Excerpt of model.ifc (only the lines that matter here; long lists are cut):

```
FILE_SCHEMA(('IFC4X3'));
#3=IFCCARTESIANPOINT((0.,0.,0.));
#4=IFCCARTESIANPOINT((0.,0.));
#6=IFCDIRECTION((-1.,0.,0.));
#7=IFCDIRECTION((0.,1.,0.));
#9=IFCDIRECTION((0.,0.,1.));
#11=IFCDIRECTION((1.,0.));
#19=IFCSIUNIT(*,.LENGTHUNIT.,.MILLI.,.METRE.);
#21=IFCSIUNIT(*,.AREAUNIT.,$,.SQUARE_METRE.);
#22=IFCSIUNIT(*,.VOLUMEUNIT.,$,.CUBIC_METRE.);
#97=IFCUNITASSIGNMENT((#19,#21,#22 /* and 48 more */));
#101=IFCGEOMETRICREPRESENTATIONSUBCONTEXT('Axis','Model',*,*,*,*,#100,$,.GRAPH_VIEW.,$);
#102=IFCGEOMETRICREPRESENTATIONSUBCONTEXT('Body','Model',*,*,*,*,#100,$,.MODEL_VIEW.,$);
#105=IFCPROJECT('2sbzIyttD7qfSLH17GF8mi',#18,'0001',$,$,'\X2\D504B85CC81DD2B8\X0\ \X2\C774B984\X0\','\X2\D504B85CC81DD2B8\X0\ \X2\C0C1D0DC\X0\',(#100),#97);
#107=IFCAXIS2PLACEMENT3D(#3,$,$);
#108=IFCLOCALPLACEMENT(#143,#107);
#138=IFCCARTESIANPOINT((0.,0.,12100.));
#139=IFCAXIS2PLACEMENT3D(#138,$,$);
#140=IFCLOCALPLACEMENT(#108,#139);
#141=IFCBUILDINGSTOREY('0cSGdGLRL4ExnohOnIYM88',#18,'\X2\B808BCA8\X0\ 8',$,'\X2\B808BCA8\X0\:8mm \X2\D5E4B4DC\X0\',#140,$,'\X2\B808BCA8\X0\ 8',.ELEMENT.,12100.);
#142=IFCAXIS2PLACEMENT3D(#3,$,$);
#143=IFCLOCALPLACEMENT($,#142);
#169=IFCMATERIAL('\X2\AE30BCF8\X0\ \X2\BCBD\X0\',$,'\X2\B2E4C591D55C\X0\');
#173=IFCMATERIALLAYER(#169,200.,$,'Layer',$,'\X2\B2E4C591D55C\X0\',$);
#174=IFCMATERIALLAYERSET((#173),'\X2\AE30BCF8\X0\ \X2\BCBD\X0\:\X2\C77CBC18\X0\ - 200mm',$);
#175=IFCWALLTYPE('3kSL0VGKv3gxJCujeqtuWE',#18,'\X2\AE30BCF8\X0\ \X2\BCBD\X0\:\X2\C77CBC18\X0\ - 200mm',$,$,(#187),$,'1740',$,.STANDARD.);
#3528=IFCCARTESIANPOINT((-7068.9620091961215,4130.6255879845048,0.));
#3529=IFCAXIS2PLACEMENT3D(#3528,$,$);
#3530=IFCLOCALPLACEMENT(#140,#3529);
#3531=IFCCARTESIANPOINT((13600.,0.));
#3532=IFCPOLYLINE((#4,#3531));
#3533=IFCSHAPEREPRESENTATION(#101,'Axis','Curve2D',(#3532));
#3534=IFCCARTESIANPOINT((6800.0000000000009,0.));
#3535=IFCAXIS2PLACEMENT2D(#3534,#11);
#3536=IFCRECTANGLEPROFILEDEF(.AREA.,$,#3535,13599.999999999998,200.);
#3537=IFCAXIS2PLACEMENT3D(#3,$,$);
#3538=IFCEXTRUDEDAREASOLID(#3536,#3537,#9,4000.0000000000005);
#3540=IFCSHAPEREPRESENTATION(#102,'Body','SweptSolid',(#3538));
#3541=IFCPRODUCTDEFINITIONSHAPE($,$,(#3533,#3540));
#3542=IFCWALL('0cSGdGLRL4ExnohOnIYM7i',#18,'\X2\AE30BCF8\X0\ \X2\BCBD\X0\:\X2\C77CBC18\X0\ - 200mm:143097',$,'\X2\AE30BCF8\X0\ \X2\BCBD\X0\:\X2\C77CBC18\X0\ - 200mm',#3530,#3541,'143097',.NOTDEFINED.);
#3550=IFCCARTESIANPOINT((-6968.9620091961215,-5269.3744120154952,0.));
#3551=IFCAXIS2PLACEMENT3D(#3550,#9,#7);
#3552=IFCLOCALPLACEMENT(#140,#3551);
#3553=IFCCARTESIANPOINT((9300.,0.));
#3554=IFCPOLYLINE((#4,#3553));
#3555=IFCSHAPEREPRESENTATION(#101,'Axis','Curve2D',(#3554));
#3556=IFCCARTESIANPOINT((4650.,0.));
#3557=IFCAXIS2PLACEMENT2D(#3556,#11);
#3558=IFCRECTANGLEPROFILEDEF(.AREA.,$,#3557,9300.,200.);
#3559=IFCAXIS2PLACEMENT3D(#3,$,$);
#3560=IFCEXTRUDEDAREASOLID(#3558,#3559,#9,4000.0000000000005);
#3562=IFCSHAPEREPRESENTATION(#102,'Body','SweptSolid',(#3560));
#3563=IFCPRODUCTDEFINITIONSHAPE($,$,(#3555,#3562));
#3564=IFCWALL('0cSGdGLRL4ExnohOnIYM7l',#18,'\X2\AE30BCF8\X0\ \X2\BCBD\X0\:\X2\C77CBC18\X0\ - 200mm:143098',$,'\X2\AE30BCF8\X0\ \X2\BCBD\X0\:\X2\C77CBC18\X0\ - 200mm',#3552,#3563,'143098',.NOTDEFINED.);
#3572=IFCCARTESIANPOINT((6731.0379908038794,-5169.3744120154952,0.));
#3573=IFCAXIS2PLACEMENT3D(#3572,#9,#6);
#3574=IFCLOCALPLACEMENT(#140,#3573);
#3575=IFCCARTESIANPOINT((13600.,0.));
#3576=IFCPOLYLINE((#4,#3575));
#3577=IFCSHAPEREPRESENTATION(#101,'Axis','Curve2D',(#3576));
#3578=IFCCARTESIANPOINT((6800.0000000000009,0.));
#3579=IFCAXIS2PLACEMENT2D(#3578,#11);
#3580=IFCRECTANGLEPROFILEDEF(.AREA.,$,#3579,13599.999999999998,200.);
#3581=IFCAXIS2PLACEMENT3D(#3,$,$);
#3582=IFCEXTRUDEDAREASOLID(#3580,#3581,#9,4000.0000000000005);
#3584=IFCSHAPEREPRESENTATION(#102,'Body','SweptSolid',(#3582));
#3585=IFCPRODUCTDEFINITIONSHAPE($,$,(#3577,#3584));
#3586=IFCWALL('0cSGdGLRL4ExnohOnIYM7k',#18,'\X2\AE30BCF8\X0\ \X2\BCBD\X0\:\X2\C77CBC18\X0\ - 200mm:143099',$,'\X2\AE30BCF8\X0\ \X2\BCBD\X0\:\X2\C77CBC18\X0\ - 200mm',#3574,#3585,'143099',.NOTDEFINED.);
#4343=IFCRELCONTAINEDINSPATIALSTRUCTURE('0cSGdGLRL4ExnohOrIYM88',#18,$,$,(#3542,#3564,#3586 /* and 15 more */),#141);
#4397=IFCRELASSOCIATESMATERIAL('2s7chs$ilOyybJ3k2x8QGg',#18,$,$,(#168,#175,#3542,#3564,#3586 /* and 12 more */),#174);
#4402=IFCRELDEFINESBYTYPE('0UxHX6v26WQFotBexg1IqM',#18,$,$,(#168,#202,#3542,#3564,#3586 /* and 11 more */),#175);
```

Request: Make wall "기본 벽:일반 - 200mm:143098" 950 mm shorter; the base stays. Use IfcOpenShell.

```python
import ifcopenshell
import ifcopenshell.geom
import ifcopenshell.util.representation
import ifcopenshell.util.shape
import ifcopenshell.util.unit

model = ifcopenshell.open("model.ifc")
unit_scale = ifcopenshell.util.unit.calculate_unit_scale(model)
settings = ifcopenshell.geom.settings()


def volume(element):
    """Net volume in cubic metres, openings subtracted."""
    shape = ifcopenshell.geom.create_shape(settings, element)
    return ifcopenshell.util.shape.get_volume(shape.geometry)


wall = model.by_guid("0cSGdGLRL4ExnohOnIYM7l")
before = volume(wall)

body = ifcopenshell.util.representation.get_representation(wall, "Model", "Body")
solid = body.Items[0]
old_height = solid.Depth
solid.Depth -= 0.95 / unit_scale
after = volume(wall)

print(f"height {old_height:g} -> {solid.Depth:g}, volume {before:.3f} -> {after:.3f} m3")

model.write("model_v2.ifc")
```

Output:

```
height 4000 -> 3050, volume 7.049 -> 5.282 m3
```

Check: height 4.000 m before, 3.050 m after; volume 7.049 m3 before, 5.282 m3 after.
